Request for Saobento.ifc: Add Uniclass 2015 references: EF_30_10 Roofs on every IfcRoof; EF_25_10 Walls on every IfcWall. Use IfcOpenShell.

First a look at what the model holds.

```python
import ifcopenshell

model = ifcopenshell.open("Saobento.ifc")
print(model.schema)
print("classifications:", [c.Name for c in model.by_type("IfcClassification")])
for ifc_class in ("IfcDoor", "IfcRoof", "IfcStair", "IfcWall", "IfcWindow"):
    print(ifc_class, len(model.by_type(ifc_class)))
```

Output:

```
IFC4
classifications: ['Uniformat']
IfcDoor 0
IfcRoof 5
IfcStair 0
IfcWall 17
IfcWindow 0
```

```python
import ifcopenshell
import ifcopenshell.api.classification

model = ifcopenshell.open("Saobento.ifc")

system = ifcopenshell.api.classification.add_classification(model, classification="Uniclass 2015")

codes = {
    "IfcRoof": ("EF_30_10", "Roofs"),
    "IfcWall": ("EF_25_10", "Walls"),
}
for ifc_class, (code, name) in codes.items():
    products = model.by_type(ifc_class)
    ifcopenshell.api.classification.add_reference(
        model, products=products, classification=system, identification=code, name=name
    )
    print(code, len(products))

model.write("Saobento_edited.ifc")
```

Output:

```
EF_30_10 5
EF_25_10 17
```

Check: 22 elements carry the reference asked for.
